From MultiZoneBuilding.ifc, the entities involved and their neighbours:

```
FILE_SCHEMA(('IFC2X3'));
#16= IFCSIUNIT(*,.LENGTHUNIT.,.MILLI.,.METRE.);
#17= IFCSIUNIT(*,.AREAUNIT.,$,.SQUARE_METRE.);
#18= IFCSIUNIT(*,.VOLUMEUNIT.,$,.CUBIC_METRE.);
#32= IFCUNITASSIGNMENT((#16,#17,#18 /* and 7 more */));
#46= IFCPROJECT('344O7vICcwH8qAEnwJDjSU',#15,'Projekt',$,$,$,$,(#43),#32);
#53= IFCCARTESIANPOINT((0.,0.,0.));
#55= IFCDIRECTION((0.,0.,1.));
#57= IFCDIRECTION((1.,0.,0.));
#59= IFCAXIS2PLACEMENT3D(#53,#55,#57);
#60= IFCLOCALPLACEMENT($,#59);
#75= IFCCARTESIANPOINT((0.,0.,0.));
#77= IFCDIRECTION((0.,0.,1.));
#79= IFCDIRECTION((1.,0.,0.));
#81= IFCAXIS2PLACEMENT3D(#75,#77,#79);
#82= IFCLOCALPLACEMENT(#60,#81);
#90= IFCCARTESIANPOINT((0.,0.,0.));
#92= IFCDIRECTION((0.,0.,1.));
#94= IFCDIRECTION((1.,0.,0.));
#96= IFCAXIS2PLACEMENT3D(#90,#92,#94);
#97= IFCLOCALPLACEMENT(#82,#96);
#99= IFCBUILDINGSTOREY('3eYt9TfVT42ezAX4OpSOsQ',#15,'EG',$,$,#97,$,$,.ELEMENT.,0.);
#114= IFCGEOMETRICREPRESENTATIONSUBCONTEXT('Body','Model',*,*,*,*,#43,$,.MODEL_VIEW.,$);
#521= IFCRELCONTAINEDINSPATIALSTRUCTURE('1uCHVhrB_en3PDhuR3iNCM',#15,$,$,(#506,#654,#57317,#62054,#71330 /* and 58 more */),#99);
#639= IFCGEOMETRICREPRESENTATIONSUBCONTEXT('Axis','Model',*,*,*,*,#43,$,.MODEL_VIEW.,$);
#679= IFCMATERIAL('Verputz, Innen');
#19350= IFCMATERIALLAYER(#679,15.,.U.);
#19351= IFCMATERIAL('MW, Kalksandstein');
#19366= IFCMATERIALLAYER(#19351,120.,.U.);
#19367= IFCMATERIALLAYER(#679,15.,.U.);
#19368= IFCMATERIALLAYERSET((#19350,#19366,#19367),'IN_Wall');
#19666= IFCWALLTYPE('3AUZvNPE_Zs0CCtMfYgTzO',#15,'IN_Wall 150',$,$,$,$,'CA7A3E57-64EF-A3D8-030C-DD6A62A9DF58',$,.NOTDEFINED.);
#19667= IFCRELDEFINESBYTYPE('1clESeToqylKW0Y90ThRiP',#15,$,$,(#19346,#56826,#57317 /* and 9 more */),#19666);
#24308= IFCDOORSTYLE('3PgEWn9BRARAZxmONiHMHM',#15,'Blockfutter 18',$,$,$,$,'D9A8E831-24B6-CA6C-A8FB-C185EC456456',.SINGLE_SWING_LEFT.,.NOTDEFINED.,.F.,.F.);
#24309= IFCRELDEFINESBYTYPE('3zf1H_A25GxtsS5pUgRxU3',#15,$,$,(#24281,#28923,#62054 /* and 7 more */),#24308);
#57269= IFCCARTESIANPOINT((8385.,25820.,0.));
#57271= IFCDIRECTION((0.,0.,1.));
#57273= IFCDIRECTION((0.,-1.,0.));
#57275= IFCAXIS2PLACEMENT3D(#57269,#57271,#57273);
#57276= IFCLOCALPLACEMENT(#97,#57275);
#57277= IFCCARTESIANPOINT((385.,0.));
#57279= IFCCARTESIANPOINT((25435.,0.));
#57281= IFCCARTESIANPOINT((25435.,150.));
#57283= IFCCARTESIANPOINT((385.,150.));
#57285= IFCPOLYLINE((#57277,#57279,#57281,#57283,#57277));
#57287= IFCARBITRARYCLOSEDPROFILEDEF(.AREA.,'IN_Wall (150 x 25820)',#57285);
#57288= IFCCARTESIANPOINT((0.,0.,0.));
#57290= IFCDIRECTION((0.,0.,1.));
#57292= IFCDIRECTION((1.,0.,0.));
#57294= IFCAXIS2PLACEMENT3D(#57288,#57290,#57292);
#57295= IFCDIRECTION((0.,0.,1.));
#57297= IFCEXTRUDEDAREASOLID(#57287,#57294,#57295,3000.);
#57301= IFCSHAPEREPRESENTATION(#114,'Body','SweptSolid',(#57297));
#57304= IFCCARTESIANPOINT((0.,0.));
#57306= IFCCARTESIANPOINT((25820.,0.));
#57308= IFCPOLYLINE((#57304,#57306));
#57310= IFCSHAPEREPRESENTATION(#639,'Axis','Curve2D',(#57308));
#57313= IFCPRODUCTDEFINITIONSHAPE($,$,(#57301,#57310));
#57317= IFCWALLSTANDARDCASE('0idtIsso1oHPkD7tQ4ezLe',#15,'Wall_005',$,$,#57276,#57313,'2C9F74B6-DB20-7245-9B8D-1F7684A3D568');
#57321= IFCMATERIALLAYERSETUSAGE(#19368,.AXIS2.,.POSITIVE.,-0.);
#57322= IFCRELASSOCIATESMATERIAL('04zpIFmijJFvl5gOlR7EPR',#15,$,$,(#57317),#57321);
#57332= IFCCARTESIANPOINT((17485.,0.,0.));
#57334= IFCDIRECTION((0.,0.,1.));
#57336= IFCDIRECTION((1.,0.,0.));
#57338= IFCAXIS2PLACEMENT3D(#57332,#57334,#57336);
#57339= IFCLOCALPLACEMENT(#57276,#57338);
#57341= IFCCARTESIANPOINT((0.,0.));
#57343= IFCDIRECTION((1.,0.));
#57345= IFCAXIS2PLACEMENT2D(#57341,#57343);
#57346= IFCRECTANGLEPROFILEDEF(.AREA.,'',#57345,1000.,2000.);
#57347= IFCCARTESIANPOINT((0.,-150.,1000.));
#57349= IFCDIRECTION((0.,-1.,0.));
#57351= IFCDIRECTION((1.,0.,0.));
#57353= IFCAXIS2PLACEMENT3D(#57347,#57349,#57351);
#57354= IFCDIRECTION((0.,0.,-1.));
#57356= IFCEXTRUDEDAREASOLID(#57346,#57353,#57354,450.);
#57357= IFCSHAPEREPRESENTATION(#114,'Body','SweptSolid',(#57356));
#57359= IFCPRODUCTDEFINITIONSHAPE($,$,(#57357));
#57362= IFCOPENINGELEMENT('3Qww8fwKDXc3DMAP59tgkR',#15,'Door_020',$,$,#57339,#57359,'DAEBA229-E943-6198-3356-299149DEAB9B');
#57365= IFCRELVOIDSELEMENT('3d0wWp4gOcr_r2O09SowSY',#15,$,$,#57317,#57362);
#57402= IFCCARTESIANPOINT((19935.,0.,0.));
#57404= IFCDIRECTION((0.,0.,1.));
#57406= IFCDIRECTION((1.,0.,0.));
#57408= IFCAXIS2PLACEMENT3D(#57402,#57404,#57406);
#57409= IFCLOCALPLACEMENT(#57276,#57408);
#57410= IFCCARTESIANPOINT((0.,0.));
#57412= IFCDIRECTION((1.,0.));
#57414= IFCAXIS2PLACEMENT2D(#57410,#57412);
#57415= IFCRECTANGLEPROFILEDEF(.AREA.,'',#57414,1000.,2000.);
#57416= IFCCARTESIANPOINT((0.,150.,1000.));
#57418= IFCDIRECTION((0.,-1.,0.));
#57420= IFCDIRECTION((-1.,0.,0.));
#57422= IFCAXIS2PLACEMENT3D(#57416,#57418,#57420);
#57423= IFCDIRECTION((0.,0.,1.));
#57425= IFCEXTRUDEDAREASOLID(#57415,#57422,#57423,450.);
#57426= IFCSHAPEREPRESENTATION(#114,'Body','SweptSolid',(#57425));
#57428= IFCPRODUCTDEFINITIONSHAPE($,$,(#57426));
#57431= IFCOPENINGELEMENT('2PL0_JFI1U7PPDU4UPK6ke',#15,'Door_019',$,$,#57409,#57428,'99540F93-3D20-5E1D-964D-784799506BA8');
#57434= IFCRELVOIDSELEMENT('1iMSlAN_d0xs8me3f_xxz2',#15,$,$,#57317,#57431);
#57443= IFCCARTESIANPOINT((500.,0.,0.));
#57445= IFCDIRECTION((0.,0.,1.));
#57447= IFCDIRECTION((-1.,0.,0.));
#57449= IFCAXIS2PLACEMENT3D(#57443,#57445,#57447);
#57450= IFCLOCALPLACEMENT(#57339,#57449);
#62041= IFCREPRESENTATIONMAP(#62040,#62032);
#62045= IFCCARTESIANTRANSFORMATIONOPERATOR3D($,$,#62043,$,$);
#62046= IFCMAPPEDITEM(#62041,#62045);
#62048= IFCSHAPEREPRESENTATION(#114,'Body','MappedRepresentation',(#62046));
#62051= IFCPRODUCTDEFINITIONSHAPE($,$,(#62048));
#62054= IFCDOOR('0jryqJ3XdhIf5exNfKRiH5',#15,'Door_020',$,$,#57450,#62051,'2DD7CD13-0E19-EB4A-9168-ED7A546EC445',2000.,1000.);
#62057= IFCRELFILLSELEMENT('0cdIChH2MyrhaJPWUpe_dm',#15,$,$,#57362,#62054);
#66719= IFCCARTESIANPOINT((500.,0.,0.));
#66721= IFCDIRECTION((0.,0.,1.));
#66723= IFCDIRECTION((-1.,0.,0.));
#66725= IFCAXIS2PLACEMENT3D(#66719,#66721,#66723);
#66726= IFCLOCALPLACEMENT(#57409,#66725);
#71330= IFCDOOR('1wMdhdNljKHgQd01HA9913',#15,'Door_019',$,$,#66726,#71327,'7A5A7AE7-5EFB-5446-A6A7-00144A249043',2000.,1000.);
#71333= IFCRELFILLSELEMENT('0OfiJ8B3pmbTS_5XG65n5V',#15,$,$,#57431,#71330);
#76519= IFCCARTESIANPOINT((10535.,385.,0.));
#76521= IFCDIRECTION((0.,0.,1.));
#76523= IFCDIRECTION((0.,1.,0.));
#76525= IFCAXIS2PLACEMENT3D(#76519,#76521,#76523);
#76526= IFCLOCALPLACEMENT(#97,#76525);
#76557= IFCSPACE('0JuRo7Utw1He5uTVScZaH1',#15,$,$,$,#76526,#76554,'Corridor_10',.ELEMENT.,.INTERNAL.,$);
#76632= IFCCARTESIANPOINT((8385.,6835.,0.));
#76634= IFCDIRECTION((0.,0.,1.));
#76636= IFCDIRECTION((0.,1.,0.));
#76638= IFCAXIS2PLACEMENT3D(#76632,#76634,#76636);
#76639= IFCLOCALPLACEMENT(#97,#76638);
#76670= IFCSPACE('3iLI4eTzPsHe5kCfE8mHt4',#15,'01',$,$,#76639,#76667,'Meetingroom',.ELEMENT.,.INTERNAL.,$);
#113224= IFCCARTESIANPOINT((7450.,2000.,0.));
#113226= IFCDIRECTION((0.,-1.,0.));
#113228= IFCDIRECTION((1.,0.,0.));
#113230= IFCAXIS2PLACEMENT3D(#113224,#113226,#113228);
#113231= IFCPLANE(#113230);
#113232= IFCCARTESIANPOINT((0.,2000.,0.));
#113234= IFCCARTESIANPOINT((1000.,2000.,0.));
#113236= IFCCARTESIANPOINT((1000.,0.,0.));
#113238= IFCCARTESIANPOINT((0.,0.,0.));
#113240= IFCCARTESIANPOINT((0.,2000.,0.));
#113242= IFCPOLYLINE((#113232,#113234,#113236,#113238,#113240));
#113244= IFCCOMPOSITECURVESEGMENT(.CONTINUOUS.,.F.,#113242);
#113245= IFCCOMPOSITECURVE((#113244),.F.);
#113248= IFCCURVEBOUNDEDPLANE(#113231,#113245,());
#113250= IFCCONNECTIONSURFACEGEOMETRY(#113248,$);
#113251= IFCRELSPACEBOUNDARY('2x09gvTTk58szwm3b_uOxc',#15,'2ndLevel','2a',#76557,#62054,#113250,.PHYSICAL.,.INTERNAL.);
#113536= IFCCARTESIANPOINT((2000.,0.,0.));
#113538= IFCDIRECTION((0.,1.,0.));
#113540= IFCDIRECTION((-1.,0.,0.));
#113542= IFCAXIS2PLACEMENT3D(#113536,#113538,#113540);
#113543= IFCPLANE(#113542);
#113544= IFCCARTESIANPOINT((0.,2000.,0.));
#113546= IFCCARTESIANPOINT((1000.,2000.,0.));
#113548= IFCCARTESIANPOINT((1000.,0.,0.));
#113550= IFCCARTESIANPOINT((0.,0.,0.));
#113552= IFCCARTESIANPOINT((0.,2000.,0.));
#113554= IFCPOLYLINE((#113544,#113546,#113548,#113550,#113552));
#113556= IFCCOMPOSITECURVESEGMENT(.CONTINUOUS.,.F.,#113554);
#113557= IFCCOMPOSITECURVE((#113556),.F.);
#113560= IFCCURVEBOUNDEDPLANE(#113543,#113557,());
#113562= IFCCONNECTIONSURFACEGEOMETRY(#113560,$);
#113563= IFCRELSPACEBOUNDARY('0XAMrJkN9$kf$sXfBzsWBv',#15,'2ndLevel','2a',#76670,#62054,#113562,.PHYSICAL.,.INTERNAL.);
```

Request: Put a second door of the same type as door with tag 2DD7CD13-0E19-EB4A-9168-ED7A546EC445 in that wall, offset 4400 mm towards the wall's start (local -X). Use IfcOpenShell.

```python
import numpy as np
import ifcopenshell
import ifcopenshell.api.feature
import ifcopenshell.api.geometry
import ifcopenshell.api.root
import ifcopenshell.geom
import ifcopenshell.util.element
import ifcopenshell.util.placement
import ifcopenshell.util.shape

model = ifcopenshell.open("MultiZoneBuilding.ifc")
settings = ifcopenshell.geom.settings()


def volume(element):
    """Net volume in cubic metres, openings subtracted."""
    shape = ifcopenshell.geom.create_shape(settings, element)
    return ifcopenshell.util.shape.get_volume(shape.geometry)


def reuse_history(source, copy):
    """copy_class also copies each property set's owner history, people and application; keep the originals."""
    for rel in copy.IsDefinedBy:
        if rel.is_a("IfcRelDefinesByProperties") and (history := rel.RelatingPropertyDefinition.OwnerHistory):
            rel.RelatingPropertyDefinition.OwnerHistory = source.OwnerHistory
            ifcopenshell.util.element.remove_deep2(model, history)


door = model.by_guid("0jryqJ3XdhIf5exNfKRiH5")
opening = door.FillsVoids[0].RelatingOpeningElement
wall = opening.VoidsElements[0].RelatingBuildingElement
before = volume(wall)
shift = ifcopenshell.util.placement.get_local_placement(wall.ObjectPlacement)[:3, 0] * -4400.0

# copy_class copies the void relationship, type, container and properties, but no geometry.
new_opening = ifcopenshell.api.root.copy_class(model, product=opening)
new_opening.Representation = ifcopenshell.util.element.copy_deep(
    model, opening.Representation, exclude=["IfcGeometricRepresentationContext", "IfcRepresentationMap"]
)
new_opening.Tag = None
new_door = ifcopenshell.api.root.copy_class(model, product=door)
new_door.Representation = ifcopenshell.util.element.copy_deep(
    model, door.Representation, exclude=["IfcGeometricRepresentationContext", "IfcRepresentationMap"]
)
new_door.Tag = None
reuse_history(door, new_door)
fills = ifcopenshell.api.feature.add_filling(model, opening=new_opening, element=new_door)
fills.OwnerHistory = new_door.OwnerHistory  # required in IFC2X3

for old, new in ((opening, new_opening), (door, new_door)):
    matrix = ifcopenshell.util.placement.get_local_placement(old.ObjectPlacement)
    matrix[:3, 3] += shift
    ifcopenshell.api.geometry.edit_object_placement(model, product=new, matrix=matrix, is_si=False)

# The copied space boundaries still share their surfaces with the original.
for rel in new_door.ProvidesBoundaries:
    if rel.ConnectionGeometry:
        rel.ConnectionGeometry = ifcopenshell.util.element.copy_deep(model, rel.ConnectionGeometry)

# Space boundary surfaces are stored in each space's coordinates; move them too.
for rel in new_door.ProvidesBoundaries:
    if not rel.ConnectionGeometry:
        continue
    surface = rel.ConnectionGeometry.SurfaceOnRelatingElement.BasisSurface
    space_matrix = ifcopenshell.util.placement.get_local_placement(rel.RelatingSpace.ObjectPlacement)
    point = np.array(surface.Position.Location.Coordinates) + space_matrix[:3, :3].T @ shift
    surface.Position = model.createIfcAxis2Placement3D(
        model.createIfcCartesianPoint(point.tolist()), surface.Position.Axis, surface.Position.RefDirection
    )

after = volume(wall)

print(f"wall volume {before:.3f} -> {after:.3f} m3")

model.write("MultiZoneBuilding_rev.ifc")
```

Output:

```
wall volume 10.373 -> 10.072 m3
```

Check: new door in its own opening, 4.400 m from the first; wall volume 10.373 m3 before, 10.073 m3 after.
